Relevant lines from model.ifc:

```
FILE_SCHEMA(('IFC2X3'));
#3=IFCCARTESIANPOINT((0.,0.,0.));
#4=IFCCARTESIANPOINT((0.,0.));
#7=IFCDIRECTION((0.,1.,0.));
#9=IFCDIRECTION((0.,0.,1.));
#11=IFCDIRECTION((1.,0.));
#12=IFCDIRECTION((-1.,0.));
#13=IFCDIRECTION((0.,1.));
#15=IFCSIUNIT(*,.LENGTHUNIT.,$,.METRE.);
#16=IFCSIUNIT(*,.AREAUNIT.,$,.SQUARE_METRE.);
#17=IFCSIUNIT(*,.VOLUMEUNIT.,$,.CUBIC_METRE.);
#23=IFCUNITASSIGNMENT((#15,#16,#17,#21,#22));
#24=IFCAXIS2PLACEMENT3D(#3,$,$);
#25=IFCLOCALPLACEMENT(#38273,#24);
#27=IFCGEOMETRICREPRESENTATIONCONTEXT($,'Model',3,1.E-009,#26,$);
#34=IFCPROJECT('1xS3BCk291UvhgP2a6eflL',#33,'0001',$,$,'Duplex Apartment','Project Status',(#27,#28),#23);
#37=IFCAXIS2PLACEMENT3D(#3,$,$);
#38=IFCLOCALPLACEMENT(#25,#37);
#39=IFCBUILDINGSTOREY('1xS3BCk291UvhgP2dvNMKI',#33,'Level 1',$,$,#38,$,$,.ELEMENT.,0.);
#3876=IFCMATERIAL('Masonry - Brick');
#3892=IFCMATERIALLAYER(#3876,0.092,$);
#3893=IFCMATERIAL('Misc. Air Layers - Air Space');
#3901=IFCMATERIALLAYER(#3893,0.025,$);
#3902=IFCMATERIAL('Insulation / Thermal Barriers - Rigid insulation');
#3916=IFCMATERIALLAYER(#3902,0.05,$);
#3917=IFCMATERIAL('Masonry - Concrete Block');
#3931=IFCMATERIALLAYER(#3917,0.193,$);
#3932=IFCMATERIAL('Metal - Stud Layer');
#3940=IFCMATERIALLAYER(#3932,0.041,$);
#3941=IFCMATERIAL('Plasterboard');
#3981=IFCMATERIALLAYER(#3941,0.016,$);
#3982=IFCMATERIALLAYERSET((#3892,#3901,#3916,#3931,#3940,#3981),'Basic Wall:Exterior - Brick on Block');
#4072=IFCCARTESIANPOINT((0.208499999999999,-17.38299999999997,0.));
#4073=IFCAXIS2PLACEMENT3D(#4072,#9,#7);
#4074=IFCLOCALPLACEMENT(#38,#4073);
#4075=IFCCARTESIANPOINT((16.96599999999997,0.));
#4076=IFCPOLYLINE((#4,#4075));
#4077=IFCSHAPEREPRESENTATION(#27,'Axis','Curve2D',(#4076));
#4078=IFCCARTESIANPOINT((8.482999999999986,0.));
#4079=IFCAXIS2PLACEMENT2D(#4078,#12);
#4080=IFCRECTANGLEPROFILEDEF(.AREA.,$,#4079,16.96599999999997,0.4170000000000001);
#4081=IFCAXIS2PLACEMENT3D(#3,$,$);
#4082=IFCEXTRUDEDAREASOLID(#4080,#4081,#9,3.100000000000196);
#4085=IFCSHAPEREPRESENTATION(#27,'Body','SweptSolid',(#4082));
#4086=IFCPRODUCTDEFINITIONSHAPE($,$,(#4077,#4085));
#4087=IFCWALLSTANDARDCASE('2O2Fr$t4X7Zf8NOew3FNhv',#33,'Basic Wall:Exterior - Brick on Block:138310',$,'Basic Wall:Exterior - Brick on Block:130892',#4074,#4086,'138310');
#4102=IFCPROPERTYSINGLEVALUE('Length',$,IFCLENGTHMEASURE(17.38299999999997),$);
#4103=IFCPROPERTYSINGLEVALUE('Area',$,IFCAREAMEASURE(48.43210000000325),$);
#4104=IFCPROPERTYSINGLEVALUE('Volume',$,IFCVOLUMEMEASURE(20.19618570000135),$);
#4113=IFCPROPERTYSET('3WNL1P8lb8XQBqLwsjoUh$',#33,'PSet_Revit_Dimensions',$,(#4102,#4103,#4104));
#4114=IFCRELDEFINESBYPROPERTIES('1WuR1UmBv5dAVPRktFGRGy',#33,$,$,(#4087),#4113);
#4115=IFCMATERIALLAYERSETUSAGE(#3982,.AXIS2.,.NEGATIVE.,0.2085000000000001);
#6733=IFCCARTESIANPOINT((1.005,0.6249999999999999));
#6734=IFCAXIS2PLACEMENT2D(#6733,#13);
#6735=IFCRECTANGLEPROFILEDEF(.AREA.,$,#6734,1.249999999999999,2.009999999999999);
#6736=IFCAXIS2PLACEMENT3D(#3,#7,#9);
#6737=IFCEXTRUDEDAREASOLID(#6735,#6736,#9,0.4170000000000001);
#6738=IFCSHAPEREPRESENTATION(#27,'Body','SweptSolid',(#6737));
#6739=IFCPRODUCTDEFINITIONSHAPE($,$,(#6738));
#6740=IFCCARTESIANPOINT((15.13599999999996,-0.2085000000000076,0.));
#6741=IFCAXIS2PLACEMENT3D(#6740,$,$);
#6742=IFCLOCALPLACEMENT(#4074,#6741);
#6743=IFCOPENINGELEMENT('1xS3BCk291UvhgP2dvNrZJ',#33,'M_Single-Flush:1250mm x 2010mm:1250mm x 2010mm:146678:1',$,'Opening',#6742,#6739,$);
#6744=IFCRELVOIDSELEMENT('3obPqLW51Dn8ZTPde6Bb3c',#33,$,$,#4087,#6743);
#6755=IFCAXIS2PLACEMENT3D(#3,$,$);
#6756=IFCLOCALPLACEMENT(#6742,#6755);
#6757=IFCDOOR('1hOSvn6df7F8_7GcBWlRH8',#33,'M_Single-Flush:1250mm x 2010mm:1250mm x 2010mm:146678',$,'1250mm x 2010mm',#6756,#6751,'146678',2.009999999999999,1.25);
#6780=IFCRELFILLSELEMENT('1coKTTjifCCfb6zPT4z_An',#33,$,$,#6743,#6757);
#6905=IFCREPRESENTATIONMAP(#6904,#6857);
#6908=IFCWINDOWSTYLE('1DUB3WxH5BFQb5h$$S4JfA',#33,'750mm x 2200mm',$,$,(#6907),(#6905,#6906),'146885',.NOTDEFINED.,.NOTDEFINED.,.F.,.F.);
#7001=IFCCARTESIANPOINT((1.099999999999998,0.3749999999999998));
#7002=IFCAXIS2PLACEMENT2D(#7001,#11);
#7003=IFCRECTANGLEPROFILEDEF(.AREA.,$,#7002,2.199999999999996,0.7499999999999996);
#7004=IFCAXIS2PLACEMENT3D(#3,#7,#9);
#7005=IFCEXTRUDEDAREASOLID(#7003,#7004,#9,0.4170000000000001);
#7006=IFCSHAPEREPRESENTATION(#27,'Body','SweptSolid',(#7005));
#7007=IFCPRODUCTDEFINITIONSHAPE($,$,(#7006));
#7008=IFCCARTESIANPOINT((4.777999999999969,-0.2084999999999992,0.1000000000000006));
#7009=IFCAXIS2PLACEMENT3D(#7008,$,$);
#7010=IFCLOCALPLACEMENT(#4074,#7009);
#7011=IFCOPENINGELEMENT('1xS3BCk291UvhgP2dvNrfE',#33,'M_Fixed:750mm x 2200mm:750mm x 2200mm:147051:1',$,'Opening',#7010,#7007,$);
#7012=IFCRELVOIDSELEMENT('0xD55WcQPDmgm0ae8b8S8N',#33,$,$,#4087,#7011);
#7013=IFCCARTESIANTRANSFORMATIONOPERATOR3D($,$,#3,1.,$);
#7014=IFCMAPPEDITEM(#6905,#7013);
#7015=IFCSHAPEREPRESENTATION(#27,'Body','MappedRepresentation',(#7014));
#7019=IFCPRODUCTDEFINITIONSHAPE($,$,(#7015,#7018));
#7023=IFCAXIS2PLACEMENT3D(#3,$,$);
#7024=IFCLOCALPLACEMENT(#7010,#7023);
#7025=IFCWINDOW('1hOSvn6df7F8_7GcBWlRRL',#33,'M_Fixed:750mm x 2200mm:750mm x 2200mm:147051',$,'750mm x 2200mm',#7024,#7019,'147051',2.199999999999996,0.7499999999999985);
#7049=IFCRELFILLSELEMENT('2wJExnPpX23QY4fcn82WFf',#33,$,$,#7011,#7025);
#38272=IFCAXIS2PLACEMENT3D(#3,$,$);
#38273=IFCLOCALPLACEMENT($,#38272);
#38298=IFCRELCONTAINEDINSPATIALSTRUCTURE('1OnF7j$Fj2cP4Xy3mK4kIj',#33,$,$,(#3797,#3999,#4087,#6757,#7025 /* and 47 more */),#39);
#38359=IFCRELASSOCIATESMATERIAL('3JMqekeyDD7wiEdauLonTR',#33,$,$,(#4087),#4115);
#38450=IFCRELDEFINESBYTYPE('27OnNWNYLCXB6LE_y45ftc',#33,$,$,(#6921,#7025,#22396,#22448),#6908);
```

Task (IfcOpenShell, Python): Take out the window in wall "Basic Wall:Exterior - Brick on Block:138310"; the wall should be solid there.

```python
import ifcopenshell
import ifcopenshell.api.feature
import ifcopenshell.api.pset
import ifcopenshell.api.root
import ifcopenshell.geom
import ifcopenshell.util.element
import ifcopenshell.util.shape
import ifcopenshell.util.unit

model = ifcopenshell.open("model.ifc")
area_scale = ifcopenshell.util.unit.calculate_unit_scale(model, "AREAUNIT")
volume_scale = ifcopenshell.util.unit.calculate_unit_scale(model, "VOLUMEUNIT")
settings = ifcopenshell.geom.settings()


def volume(element):
    """Net volume in cubic metres, openings subtracted."""
    shape = ifcopenshell.geom.create_shape(settings, element)
    return ifcopenshell.util.shape.get_volume(shape.geometry)


window = model.by_id(7025)
opening = window.FillsVoids[0].RelatingOpeningElement
wall = opening.VoidsElements[0].RelatingBuildingElement
before = volume(wall)

ifcopenshell.api.root.remove_product(model, product=window)
ifcopenshell.api.feature.remove_feature(model, feature=opening)

after = volume(wall)
thickness = 0.417  # wall thickness in metres

# Update the wall's stored quantities.
pset = model.by_id(ifcopenshell.util.element.get_pset(wall, "PSet_Revit_Dimensions", should_inherit=False)["id"])
ifcopenshell.api.pset.edit_pset(model, pset=pset, properties={
    "Area": model.create_entity("IfcAreaMeasure", after / thickness / area_scale),
    "Volume": model.create_entity("IfcVolumeMeasure", after / volume_scale),
})

print(f"wall volume {before:.3f} -> {after:.3f} m3")

model.write("model_rev.ifc")
```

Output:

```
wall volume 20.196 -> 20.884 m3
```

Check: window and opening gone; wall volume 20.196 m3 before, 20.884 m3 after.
